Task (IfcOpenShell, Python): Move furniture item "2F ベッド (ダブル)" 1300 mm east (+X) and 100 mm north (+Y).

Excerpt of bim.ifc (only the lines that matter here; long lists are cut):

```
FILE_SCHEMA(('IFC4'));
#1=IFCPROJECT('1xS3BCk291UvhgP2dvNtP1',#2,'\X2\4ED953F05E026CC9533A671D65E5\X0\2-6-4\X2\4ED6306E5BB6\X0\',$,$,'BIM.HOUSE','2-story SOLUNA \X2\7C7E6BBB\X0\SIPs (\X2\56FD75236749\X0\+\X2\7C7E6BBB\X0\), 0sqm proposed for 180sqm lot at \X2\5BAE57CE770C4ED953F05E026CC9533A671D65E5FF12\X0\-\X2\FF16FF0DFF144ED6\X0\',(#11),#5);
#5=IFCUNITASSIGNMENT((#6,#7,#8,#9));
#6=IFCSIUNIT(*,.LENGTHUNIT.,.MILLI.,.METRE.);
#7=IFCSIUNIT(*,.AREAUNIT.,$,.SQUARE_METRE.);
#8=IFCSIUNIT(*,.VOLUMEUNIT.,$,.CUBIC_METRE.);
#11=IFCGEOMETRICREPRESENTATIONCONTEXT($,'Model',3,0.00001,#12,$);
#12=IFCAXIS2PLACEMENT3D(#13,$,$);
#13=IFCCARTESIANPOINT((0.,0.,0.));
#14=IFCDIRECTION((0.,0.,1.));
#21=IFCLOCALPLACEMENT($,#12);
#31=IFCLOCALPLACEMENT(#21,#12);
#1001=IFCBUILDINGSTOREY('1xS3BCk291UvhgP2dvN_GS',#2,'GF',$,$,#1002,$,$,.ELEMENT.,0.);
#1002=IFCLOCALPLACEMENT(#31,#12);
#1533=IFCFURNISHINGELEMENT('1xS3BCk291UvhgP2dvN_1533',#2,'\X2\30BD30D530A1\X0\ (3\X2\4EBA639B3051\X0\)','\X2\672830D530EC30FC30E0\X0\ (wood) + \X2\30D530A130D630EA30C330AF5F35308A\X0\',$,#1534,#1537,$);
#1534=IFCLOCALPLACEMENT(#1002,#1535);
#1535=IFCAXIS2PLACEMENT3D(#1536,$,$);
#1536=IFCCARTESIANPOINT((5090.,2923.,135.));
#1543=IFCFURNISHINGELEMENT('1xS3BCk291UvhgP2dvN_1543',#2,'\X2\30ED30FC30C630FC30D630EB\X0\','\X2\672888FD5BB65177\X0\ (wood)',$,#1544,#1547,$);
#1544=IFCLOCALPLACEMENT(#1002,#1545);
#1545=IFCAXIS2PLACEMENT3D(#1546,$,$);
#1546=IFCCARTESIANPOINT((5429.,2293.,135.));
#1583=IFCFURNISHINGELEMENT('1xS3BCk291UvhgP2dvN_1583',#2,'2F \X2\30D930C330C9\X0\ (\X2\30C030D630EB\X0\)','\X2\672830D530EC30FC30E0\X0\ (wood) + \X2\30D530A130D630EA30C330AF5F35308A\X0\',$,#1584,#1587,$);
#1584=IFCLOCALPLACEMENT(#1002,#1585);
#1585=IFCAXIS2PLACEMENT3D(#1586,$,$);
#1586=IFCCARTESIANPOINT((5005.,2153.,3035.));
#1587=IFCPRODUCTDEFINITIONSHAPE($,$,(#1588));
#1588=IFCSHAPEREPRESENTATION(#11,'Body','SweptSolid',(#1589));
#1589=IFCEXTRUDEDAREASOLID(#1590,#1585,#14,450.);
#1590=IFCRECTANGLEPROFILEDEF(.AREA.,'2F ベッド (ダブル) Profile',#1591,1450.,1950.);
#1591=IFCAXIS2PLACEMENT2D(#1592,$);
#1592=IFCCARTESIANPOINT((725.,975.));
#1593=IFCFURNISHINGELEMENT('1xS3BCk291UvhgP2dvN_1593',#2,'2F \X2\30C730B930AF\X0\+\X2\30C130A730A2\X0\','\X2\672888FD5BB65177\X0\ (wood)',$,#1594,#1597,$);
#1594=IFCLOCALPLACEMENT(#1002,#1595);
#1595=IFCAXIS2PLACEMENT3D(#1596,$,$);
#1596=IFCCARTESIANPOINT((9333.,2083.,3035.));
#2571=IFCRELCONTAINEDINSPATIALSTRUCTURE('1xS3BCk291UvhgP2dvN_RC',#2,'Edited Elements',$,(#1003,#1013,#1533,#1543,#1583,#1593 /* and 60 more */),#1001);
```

```python
import ifcopenshell
import ifcopenshell.api.geometry
import ifcopenshell.util.placement
import ifcopenshell.util.unit

model = ifcopenshell.open("bim.ifc")
unit_scale = ifcopenshell.util.unit.calculate_unit_scale(model)

item = model.by_guid("1xS3BCk291UvhgP2dvN_1583")
matrix = ifcopenshell.util.placement.get_local_placement(item.ObjectPlacement)
matrix[0, 3] += 1.3 / unit_scale
matrix[1, 3] += 0.1 / unit_scale
ifcopenshell.api.geometry.edit_object_placement(model, product=item, matrix=matrix, is_si=False)

print(ifcopenshell.util.placement.get_local_placement(item.ObjectPlacement).round(3) + 0.0)

model.write("bim_edited.ifc")
```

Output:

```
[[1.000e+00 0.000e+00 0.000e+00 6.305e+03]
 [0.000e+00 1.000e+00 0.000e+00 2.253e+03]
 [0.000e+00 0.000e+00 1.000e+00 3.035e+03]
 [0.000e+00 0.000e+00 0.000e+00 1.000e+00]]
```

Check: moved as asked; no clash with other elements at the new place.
